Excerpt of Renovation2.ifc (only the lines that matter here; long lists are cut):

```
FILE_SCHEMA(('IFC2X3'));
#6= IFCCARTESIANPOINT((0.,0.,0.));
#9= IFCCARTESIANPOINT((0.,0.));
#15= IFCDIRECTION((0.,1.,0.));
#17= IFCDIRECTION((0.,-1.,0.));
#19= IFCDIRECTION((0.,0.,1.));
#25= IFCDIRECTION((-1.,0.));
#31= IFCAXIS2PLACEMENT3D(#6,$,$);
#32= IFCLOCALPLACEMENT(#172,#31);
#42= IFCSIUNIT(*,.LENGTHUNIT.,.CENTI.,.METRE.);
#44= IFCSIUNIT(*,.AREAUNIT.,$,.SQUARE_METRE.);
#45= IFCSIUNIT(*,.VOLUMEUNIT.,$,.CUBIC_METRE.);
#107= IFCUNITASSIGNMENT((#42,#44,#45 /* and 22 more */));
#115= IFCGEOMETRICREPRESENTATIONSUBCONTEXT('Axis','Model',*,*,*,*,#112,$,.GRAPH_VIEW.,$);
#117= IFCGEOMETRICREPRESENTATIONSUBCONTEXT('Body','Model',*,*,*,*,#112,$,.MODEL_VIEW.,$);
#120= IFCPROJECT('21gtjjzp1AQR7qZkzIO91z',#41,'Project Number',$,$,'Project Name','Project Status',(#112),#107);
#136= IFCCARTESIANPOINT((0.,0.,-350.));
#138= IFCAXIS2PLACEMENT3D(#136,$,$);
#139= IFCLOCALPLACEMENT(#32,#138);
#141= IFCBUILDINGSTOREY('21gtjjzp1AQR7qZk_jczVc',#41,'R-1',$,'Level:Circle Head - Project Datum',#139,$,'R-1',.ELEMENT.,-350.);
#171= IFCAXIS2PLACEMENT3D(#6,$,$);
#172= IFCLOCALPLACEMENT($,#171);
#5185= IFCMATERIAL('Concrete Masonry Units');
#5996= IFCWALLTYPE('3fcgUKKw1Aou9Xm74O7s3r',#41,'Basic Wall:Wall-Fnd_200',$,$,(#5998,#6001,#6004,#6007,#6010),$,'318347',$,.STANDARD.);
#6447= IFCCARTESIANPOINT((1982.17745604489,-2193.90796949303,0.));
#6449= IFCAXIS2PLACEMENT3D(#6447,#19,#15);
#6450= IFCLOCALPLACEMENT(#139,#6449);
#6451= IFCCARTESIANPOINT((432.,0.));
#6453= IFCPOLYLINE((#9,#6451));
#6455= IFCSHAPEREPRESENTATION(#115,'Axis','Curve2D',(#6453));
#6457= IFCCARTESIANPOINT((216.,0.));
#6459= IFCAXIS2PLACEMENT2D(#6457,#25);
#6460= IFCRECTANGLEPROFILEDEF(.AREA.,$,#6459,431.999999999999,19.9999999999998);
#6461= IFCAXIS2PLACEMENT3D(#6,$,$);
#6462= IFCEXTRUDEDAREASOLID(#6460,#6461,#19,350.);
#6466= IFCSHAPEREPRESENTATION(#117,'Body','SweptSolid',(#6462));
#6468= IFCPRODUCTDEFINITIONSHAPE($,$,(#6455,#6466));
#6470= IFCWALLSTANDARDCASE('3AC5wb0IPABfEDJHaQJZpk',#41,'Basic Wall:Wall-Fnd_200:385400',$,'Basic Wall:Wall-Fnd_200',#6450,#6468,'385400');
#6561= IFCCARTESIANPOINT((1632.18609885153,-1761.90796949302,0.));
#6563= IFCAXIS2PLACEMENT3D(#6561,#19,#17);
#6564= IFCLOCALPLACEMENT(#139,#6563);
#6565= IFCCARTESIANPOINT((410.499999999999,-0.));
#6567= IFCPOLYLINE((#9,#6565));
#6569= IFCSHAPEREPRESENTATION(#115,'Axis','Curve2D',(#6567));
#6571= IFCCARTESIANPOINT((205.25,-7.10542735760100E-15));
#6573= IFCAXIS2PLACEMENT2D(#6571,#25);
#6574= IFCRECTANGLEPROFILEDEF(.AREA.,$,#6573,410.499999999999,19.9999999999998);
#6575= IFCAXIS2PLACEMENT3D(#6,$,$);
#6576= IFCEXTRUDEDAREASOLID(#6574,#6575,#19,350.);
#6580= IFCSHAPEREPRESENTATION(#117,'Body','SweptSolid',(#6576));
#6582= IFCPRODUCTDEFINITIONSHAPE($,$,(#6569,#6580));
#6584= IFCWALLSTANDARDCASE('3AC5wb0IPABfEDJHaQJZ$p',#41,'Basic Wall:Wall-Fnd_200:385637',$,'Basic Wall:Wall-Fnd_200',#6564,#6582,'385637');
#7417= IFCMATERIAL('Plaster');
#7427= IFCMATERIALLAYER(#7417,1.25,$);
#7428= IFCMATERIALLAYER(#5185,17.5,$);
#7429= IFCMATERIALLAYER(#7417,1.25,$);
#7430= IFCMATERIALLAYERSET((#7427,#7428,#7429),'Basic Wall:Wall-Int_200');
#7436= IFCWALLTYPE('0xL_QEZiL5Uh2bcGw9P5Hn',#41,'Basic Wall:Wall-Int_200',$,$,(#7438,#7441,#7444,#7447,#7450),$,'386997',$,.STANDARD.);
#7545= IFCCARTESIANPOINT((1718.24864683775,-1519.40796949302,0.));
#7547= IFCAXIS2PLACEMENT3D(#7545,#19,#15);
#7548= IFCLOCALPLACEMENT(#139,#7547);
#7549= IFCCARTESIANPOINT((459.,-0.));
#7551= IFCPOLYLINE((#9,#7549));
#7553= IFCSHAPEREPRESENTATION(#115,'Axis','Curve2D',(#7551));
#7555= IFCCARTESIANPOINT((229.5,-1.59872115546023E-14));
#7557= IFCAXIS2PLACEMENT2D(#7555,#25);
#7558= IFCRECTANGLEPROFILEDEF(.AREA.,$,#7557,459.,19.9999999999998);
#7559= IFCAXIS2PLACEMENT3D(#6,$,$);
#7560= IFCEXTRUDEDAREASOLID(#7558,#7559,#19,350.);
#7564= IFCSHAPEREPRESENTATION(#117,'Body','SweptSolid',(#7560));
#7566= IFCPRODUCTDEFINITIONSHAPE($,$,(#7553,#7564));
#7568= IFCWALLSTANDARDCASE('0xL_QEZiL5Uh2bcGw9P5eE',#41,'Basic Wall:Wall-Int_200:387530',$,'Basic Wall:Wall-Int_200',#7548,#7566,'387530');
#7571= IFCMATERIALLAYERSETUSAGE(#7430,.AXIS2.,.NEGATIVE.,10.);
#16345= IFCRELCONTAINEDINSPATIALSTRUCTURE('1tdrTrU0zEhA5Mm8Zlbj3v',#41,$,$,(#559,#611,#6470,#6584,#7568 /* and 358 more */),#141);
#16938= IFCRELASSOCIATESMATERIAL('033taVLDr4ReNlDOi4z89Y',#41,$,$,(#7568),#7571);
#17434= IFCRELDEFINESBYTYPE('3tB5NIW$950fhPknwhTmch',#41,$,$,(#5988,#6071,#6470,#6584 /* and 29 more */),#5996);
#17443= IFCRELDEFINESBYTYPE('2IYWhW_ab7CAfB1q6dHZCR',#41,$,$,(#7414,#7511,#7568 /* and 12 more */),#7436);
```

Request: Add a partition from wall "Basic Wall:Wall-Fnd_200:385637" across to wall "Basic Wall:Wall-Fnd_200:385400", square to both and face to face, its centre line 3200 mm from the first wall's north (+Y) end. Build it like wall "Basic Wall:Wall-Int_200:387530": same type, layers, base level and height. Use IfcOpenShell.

```python
import numpy as np
import ifcopenshell
import ifcopenshell.api.geometry
import ifcopenshell.api.material
import ifcopenshell.api.pset
import ifcopenshell.api.root
import ifcopenshell.api.spatial
import ifcopenshell.api.type
import ifcopenshell.geom
import ifcopenshell.util.element
import ifcopenshell.util.placement
import ifcopenshell.util.representation
import ifcopenshell.util.shape
import ifcopenshell.util.unit

model = ifcopenshell.open("Renovation2.ifc")
unit_scale = ifcopenshell.util.unit.calculate_unit_scale(model)
settings = ifcopenshell.geom.settings()
settings.set("use-world-coords", True)

start_wall = model.by_id(6584)
end_wall = model.by_id(6470)
like = model.by_id(7568)
matrix = ifcopenshell.util.placement.get_local_placement(start_wall.ObjectPlacement)
matrix[:3, 3] *= unit_scale


def extent(element):
    """Bounding box in the first wall's axes, in metres."""
    shape = ifcopenshell.geom.create_shape(settings, element)
    points = (ifcopenshell.util.shape.get_vertices(shape.geometry) - matrix[:3, 3]) @ matrix[:3, :3]
    return points.min(axis=0), points.max(axis=0)


y_start = extent(start_wall)[1][1]
y_end = extent(end_wall)[0][1]
like_min, like_max = extent(like)
length, height = float(abs(y_end - y_start)), float(like_max[2] - like_min[2])
layer_set = ifcopenshell.util.element.get_material(like, should_skip_usage=True)
thickness = sum(layer.LayerThickness for layer in layer_set.MaterialLayers) * unit_scale

wall = ifcopenshell.api.root.create_entity(model, ifc_class="IfcWallStandardCase", name="New partition")
storey = ifcopenshell.util.element.get_container(like)
ifcopenshell.api.spatial.assign_container(model, products=[wall], relating_structure=storey)
ifcopenshell.api.type.assign_type(
    model, related_objects=[wall], relating_type=ifcopenshell.util.element.get_type(like), should_map_representations=False
)
rel = ifcopenshell.api.material.assign_material(
    model, products=[wall], type="IfcMaterialLayerSetUsage", material=layer_set
)
rel.RelatingMaterial.OffsetFromReferenceLine = -thickness / 2 / unit_scale
pset = ifcopenshell.api.pset.add_pset(model, product=wall, name="Pset_WallCommon")
ifcopenshell.api.pset.edit_pset(model, pset=pset, properties={"IsExternal": False, "LoadBearing": False})

# The axis runs down the middle of the wall.
axis = ifcopenshell.api.geometry.add_axis_representation(
    model, context=ifcopenshell.util.representation.get_context(model, "Model", "Axis"), axis=[(0.0, 0.0), (length, 0.0)]
)
body = ifcopenshell.api.geometry.add_wall_representation(
    model,
    context=ifcopenshell.util.representation.get_context(model, "Model", "Body", "MODEL_VIEW"),
    length=length,
    height=height,
    thickness=thickness,
    offset=-thickness / 2,
)
for representation in (axis, body):
    ifcopenshell.api.geometry.assign_representation(model, product=wall, representation=representation)

placement = matrix @ ifcopenshell.util.placement.rotation(90, "Z")
placement[:, 3] = matrix @ np.array([extent(start_wall)[0][0] + 3.2, y_start, like_min[2], 1.0])
ifcopenshell.api.geometry.edit_object_placement(model, product=wall, matrix=placement)

print(f"partition {length:.3f} m long, {height:.3f} m high, {thickness:.3f} m thick")

model.write("Renovation2_v2.ifc")
```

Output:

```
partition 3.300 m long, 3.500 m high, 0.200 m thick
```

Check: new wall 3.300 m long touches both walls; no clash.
